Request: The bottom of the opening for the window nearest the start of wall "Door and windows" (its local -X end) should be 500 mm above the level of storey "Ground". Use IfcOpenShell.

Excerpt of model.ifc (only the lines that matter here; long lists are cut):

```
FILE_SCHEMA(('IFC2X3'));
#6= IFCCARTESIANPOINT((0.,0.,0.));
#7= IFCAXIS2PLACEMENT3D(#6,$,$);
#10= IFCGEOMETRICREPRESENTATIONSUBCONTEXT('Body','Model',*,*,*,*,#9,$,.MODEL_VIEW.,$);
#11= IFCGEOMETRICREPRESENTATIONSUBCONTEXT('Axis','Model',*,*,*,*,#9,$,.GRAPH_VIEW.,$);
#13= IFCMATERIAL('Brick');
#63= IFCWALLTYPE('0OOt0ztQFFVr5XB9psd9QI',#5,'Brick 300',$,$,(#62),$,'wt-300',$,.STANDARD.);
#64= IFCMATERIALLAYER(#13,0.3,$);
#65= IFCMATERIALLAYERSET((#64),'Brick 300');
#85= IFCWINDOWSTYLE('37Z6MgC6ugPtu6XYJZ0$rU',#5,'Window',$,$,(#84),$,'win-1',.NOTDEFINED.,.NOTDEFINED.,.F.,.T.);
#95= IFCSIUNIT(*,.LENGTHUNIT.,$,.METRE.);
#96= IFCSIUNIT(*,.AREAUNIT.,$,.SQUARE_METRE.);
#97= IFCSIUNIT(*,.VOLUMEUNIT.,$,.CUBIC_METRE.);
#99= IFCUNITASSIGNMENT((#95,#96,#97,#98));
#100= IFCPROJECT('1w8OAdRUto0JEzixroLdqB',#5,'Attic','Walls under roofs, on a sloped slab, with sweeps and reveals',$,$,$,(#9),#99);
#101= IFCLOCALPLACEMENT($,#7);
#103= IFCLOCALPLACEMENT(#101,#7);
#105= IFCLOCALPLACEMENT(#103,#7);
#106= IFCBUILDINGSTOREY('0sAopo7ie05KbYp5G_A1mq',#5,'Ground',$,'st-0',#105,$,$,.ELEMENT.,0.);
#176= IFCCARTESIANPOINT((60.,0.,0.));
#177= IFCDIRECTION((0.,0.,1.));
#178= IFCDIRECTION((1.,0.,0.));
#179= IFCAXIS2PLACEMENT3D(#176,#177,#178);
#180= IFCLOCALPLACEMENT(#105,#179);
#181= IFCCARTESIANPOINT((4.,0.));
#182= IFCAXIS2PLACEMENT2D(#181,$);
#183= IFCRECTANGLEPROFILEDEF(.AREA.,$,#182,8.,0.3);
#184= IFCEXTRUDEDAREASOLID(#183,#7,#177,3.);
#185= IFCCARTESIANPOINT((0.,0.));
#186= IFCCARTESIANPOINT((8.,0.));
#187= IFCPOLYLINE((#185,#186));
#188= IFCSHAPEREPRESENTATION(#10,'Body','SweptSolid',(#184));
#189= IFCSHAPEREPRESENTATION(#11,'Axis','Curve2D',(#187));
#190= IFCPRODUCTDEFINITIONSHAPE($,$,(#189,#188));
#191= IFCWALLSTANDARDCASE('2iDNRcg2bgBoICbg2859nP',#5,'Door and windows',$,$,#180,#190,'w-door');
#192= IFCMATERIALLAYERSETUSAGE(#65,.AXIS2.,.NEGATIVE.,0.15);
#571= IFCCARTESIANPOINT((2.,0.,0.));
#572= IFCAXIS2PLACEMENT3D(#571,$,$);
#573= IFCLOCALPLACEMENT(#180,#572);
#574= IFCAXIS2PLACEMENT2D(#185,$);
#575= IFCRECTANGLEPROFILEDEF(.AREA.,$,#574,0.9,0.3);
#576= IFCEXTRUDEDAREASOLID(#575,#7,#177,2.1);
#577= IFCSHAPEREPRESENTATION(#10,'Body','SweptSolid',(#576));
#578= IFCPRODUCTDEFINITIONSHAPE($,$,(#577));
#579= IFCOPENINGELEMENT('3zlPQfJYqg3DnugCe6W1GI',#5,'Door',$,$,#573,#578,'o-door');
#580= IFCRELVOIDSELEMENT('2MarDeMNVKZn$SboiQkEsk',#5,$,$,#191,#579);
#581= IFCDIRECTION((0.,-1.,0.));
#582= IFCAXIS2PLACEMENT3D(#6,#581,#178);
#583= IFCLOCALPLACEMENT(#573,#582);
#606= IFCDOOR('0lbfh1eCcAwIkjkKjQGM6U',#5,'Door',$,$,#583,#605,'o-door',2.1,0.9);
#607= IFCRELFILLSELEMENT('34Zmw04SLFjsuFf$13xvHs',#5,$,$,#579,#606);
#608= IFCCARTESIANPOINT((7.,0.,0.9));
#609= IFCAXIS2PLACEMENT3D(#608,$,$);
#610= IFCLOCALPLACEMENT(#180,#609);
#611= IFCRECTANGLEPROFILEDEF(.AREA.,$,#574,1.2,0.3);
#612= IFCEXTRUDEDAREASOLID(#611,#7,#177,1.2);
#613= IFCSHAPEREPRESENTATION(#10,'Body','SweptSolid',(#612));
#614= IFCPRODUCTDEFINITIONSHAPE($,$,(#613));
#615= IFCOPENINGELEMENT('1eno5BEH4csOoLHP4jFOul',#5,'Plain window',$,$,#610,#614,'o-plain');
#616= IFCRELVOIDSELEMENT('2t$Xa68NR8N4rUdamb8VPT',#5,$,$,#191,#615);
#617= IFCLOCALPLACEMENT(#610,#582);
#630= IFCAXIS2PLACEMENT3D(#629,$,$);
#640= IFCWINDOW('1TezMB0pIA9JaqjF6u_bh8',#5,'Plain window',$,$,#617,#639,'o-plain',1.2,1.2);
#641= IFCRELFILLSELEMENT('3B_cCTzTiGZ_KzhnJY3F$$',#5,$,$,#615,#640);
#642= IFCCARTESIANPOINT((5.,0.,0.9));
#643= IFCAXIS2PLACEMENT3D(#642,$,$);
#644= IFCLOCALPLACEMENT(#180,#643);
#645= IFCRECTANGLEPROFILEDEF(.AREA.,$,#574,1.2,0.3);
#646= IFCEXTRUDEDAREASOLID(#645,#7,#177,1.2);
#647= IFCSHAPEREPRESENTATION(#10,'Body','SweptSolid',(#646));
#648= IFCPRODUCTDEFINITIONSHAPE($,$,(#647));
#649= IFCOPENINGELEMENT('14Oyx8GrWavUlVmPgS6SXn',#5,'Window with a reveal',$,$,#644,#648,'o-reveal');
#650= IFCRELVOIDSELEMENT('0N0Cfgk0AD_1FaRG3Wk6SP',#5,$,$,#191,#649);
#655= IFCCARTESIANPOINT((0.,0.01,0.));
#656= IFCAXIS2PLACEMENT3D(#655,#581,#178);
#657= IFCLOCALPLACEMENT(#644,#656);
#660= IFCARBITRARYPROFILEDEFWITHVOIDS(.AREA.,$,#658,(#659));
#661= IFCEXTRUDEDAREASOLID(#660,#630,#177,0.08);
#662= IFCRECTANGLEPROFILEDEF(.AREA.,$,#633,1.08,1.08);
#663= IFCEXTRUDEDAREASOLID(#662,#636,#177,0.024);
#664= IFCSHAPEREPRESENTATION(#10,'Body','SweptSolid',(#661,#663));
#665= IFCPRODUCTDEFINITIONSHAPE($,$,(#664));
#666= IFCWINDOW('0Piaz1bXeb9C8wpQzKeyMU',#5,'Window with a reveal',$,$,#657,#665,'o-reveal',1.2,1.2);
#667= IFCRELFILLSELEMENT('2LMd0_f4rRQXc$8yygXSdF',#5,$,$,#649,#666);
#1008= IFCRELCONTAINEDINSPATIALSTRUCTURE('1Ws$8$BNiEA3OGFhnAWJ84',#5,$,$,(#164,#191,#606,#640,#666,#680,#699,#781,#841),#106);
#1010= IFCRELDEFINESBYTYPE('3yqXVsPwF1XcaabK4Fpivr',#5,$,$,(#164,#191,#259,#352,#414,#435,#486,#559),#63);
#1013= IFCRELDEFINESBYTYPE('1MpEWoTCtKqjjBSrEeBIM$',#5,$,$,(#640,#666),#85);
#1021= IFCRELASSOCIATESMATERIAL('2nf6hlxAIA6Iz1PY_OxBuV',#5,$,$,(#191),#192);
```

```python
import numpy as np
import ifcopenshell
import ifcopenshell.api.geometry
import ifcopenshell.geom
import ifcopenshell.util.element
import ifcopenshell.util.placement
import ifcopenshell.util.shape
import ifcopenshell.util.unit

model = ifcopenshell.open("model.ifc")
unit_scale = ifcopenshell.util.unit.calculate_unit_scale(model)

window = model.by_guid("0Piaz1bXeb9C8wpQzKeyMU")
opening = window.FillsVoids[0].RelatingOpeningElement
storey = ifcopenshell.util.element.get_container(window, ifc_class="IfcBuildingStorey")
level = ifcopenshell.util.placement.get_local_placement(storey.ObjectPlacement)[2, 3]

# The opening's origin need not be at the sill, so measure its lowest point.
shape = ifcopenshell.geom.create_shape(ifcopenshell.geom.settings(), opening)
bottom = ifcopenshell.util.shape.get_shape_bottom_elevation(shape, shape.geometry) / unit_scale
dz = level + 0.5 - bottom

shift = np.array([0.0, 0.0, dz])
# The window is placed relative to its opening, so it follows when the opening moves.
matrix = ifcopenshell.util.placement.get_local_placement(opening.ObjectPlacement)
matrix[:3, 3] += shift
ifcopenshell.api.geometry.edit_object_placement(
    model, product=opening, matrix=matrix, is_si=False, should_transform_children=True
)

print(f"moved by {dz * unit_scale:+.3f} m")

model.write("model_rev.ifc")
```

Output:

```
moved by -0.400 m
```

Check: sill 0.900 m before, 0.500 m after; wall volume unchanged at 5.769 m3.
